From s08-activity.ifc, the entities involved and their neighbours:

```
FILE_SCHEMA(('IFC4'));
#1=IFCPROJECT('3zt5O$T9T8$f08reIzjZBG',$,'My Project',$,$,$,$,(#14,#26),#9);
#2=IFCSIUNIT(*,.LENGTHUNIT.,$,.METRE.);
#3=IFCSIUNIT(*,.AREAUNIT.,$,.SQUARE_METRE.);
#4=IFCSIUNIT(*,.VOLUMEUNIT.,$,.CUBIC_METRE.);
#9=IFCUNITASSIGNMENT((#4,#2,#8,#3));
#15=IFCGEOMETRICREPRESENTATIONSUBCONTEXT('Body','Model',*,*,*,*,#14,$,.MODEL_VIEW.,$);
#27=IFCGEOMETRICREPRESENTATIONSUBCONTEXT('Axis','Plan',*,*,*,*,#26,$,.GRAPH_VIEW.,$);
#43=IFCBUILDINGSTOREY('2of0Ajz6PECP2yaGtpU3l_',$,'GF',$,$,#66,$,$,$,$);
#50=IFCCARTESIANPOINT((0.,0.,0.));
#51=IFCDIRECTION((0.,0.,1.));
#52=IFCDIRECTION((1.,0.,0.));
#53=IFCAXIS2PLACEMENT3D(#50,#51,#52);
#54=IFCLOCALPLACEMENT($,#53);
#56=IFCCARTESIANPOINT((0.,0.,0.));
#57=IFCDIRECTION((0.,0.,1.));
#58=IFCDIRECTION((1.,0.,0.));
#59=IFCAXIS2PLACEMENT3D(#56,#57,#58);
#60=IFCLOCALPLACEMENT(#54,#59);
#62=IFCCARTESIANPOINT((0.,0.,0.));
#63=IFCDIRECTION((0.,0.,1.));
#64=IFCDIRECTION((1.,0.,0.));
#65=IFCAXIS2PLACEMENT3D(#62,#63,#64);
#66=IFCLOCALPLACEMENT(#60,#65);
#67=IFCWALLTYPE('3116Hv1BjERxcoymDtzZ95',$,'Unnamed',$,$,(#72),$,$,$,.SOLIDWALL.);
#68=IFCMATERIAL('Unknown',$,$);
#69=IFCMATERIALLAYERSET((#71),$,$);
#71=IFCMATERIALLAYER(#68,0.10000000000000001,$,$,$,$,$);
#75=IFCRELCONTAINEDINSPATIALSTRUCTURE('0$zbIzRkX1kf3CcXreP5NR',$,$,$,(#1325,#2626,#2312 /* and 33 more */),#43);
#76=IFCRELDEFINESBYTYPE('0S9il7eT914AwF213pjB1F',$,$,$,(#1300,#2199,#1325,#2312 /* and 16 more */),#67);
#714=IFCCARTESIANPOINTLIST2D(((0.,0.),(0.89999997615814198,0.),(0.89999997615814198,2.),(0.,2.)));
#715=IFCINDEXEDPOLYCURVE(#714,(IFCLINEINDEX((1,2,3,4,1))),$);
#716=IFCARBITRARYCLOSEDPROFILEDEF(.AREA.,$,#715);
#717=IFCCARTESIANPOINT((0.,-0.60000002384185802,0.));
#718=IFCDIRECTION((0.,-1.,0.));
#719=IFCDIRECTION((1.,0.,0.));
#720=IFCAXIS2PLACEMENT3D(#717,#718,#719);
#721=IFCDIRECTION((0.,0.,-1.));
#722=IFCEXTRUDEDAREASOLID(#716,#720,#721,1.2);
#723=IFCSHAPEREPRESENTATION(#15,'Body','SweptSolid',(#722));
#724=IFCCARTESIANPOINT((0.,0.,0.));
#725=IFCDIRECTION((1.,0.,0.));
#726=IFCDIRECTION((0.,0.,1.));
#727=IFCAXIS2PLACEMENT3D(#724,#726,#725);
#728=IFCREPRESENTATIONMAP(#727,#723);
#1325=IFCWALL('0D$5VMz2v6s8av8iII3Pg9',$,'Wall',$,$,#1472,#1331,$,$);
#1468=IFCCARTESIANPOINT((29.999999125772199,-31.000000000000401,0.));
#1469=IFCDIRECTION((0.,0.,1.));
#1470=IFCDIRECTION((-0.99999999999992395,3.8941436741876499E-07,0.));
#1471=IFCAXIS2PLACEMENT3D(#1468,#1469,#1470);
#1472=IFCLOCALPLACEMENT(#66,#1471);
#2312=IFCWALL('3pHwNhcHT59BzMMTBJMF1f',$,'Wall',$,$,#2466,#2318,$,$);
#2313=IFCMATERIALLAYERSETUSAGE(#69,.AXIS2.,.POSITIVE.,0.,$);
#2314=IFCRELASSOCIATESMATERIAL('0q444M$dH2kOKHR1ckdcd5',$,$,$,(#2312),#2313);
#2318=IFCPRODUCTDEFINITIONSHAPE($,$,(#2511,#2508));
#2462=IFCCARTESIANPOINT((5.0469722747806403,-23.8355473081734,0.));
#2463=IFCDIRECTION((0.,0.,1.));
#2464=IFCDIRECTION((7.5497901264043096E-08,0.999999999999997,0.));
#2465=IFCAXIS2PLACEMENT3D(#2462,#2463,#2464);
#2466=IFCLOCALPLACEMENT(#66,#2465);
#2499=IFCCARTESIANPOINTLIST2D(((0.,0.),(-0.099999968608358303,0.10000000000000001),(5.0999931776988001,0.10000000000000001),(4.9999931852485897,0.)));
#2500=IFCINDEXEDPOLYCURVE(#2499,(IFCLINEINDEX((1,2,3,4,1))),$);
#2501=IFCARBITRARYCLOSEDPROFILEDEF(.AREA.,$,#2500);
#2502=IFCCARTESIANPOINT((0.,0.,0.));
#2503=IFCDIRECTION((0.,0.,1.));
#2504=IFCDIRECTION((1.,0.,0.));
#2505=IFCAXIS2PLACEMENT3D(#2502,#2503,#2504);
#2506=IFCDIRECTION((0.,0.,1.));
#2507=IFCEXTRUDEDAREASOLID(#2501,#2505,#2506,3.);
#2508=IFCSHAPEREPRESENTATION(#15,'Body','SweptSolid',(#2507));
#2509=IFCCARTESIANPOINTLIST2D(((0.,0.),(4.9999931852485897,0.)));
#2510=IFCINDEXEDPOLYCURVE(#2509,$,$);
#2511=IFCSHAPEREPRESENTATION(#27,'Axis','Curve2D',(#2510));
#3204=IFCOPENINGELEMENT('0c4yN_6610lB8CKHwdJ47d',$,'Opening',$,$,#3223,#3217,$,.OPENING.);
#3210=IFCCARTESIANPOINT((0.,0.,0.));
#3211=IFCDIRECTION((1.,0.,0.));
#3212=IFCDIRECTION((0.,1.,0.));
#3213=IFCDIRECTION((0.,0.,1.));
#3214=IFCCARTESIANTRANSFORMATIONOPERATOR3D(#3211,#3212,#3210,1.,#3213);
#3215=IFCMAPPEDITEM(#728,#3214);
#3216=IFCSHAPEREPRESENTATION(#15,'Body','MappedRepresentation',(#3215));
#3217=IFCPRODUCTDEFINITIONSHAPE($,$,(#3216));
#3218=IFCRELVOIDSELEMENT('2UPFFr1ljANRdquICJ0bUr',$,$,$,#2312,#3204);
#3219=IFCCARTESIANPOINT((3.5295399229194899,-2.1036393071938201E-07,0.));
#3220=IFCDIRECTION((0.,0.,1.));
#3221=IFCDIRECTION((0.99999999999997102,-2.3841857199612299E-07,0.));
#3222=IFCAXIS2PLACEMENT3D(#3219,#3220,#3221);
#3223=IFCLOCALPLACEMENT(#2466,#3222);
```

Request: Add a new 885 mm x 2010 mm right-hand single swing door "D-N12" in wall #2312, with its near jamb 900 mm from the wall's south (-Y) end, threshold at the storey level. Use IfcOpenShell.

```python
import numpy as np
import ifcopenshell
import ifcopenshell.api.feature
import ifcopenshell.api.geometry
import ifcopenshell.api.root
import ifcopenshell.api.spatial
import ifcopenshell.geom
import ifcopenshell.util.element
import ifcopenshell.util.placement
import ifcopenshell.util.representation
import ifcopenshell.util.shape
import ifcopenshell.util.unit

model = ifcopenshell.open("s08-activity.ifc")
unit_scale = ifcopenshell.util.unit.calculate_unit_scale(model)
settings = ifcopenshell.geom.settings()


def volume(element):
    """Net volume in cubic metres, openings subtracted."""
    shape = ifcopenshell.geom.create_shape(settings, element)
    return ifcopenshell.util.shape.get_volume(shape.geometry)


wall = model.by_guid("3pHwNhcHT59BzMMTBJMF1f")
storey = ifcopenshell.util.element.get_container(wall, ifc_class="IfcBuildingStorey")
context = ifcopenshell.util.representation.get_context(model, "Model", "Body", "MODEL_VIEW")
before = volume(wall)

width, height, from_end, sill = 0.885, 2.01, 0.9, 0.0  # metres

# The wall runs along its own X axis, and the end named is its -X end.
wall_shape = ifcopenshell.geom.create_shape(settings, wall)
x, y, z = ifcopenshell.util.shape.get_vertices(wall_shape.geometry).T
start = x.min() + from_end
face, thickness = float(y.min()), float(y.max() - y.min())
wall_matrix = ifcopenshell.util.placement.get_local_placement(wall.ObjectPlacement)
level = ifcopenshell.util.placement.get_local_placement(storey.ObjectPlacement)[2, 3]


def in_wall(x, y):
    """Placement at x, y metres in the wall's axes, at sill height."""
    matrix = wall_matrix.copy()
    matrix[:, 3] = wall_matrix @ np.array([x / unit_scale, y / unit_scale, 0.0, 1.0])
    matrix[2, 3] = level + sill / unit_scale
    return matrix


# Opening: a box that overshoots both wall faces by 50 mm.
opening = ifcopenshell.api.root.create_entity(model, ifc_class="IfcOpeningElement", predefined_type="OPENING")
box = ifcopenshell.api.geometry.add_wall_representation(
    model, context=context, length=width, height=height, thickness=thickness + 0.1
)
ifcopenshell.api.geometry.assign_representation(model, product=opening, representation=box)
ifcopenshell.api.geometry.edit_object_placement(model, product=opening, matrix=in_wall(start, face - 0.05), is_si=False)
ifcopenshell.api.feature.add_feature(model, feature=opening, element=wall)

door = ifcopenshell.api.root.create_entity(model, ifc_class="IfcDoor", name="D-N12", predefined_type="DOOR")
door.OverallWidth, door.OverallHeight = width / unit_scale, height / unit_scale
door.OperationType = "SINGLE_SWING_RIGHT"
body = ifcopenshell.api.geometry.add_door_representation(
    model,
    context=context,
    overall_width=door.OverallWidth,
    overall_height=door.OverallHeight,
    operation_type="SINGLE_SWING_RIGHT",
    lining_properties={"LiningDepth": thickness / unit_scale, "ThresholdDepth": thickness / unit_scale},
)
ifcopenshell.api.geometry.assign_representation(model, product=door, representation=body)
ifcopenshell.api.spatial.assign_container(model, products=[door], relating_structure=storey)
ifcopenshell.api.feature.add_filling(model, opening=opening, element=door)

# The lining spans the wall, so the door starts at the wall face.
ifcopenshell.api.geometry.edit_object_placement(model, product=door, matrix=in_wall(start, face), is_si=False)

after = volume(wall)

print(f"wall volume {before:.3f} -> {after:.3f} m3")

model.write("s08-activity_updated.ifc")
```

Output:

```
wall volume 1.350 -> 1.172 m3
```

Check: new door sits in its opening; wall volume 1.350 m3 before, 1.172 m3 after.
